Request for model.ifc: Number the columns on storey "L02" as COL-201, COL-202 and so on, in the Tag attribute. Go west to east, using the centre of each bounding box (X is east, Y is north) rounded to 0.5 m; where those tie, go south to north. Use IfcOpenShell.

First a look at what the model holds.

```python
import ifcopenshell
import ifcopenshell.util.element
import ifcopenshell.util.placement

model = ifcopenshell.open("model.ifc")
print(model.schema)
storey = next(s for s in model.by_type("IfcBuildingStorey") if s.Name == "L02")
columns = [e for e in ifcopenshell.util.element.get_decomposition(storey) if e.is_a("IfcColumn")]
for e in sorted(columns, key=lambda e: e.id()):
    origin = ifcopenshell.util.placement.get_local_placement(e.ObjectPlacement)[:3, 3]
    print(e.id(), e.Tag, e.Name, origin.round(2) + 0.0, sep=" | ")
```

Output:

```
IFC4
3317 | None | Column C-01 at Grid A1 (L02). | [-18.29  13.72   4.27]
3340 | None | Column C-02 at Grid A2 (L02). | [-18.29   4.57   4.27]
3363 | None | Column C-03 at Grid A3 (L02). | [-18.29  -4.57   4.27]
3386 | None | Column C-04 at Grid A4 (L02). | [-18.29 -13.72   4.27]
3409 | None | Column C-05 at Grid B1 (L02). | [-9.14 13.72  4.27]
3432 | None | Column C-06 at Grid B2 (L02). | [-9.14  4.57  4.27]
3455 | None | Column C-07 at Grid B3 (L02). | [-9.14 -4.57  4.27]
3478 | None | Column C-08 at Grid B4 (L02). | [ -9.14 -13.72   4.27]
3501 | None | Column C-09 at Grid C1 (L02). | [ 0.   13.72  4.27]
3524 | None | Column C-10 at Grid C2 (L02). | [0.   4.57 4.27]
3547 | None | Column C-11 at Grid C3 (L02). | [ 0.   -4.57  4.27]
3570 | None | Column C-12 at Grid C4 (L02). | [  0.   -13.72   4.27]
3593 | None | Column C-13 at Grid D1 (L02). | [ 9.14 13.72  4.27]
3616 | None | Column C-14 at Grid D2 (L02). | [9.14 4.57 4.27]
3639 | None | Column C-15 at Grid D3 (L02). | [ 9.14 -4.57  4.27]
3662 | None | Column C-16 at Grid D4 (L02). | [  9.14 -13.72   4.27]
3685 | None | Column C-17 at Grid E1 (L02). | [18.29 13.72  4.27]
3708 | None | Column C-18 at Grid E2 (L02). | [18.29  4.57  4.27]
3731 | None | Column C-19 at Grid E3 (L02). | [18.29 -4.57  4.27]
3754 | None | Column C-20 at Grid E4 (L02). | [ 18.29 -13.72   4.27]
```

```python
import ifcopenshell
import ifcopenshell.geom
import ifcopenshell.util.element
import ifcopenshell.util.shape

model = ifcopenshell.open("model.ifc")
settings = ifcopenshell.geom.settings()
settings.set("use-world-coords", True)


def centre(element):
    shape = ifcopenshell.geom.create_shape(settings, element)
    return ifcopenshell.util.shape.get_bbox_centroid(shape.geometry)


storey = next(s for s in model.by_type("IfcBuildingStorey") if s.Name == "L02")
columns = [e for e in ifcopenshell.util.element.get_decomposition(storey) if e.is_a("IfcColumn")]

# Insertion points can sit at a corner or the storey origin, so sort by the geometry (in metres).
centres = {e: centre(e) for e in columns}
columns.sort(key=lambda e: (round(centres[e][0] / 0.5), centres[e][1]))

for i, e in enumerate(columns, start=1):
    number = f"COL-2{i:02d}"
    e.Tag = number
    print(e.id(), number)

model.write("model_v2.ifc")
```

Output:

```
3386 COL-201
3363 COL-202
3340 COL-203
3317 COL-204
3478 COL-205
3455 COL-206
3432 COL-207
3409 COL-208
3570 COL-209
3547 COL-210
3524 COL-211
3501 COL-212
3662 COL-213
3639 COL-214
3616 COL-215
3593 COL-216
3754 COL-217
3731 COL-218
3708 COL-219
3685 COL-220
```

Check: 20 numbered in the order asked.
